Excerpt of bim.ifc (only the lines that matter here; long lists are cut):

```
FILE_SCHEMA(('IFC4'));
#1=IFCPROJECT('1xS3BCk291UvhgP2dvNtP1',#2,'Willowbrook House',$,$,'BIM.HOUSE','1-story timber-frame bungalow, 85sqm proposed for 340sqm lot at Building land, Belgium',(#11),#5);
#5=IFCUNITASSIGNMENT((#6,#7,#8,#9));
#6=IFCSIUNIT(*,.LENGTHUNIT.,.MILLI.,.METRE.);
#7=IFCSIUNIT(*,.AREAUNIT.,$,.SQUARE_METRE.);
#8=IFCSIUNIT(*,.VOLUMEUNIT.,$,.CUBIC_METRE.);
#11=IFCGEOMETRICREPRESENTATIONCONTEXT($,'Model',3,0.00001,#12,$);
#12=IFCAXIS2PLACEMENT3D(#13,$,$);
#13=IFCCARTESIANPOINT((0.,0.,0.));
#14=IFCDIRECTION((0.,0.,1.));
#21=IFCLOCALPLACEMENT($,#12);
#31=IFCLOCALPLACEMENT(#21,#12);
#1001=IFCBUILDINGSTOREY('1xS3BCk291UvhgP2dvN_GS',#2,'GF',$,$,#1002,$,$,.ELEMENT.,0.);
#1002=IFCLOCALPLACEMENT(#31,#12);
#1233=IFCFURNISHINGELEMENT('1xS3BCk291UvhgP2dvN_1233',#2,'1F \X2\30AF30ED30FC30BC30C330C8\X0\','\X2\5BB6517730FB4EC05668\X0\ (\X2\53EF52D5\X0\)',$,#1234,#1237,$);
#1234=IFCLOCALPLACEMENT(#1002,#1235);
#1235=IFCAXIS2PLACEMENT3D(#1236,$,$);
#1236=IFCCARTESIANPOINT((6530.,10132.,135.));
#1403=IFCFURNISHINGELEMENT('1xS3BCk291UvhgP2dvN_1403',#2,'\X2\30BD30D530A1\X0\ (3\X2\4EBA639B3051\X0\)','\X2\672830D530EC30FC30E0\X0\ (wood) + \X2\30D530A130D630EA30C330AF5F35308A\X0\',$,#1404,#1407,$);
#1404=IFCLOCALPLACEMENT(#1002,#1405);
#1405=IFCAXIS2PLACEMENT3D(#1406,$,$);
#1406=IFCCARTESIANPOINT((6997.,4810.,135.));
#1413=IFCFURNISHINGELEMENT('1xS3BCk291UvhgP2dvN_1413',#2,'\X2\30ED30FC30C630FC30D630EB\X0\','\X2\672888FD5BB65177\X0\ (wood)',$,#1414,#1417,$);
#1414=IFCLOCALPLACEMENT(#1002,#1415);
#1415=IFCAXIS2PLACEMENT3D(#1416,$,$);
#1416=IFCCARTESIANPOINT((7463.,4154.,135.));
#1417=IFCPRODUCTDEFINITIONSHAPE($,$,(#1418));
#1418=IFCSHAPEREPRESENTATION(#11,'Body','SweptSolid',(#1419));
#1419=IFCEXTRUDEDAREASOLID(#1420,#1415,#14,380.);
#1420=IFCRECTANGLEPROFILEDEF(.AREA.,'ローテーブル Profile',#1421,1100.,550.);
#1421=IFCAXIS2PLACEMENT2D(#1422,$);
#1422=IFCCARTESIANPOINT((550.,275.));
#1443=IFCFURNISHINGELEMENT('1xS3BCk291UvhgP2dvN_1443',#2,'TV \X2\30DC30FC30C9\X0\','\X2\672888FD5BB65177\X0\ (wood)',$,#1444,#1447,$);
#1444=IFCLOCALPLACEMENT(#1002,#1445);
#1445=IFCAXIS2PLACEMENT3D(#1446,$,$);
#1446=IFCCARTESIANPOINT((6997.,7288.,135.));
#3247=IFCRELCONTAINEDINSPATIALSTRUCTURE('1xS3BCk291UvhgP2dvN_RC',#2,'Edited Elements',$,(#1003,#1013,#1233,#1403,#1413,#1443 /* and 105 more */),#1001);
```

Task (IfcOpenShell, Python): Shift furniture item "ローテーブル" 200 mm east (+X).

```python
import ifcopenshell
import ifcopenshell.api.geometry
import ifcopenshell.util.placement

model = ifcopenshell.open("bim.ifc")

item = model.by_id(1413)
matrix = ifcopenshell.util.placement.get_local_placement(item.ObjectPlacement)
matrix[0, 3] += 200.0
ifcopenshell.api.geometry.edit_object_placement(model, product=item, matrix=matrix, is_si=False)

print(ifcopenshell.util.placement.get_local_placement(item.ObjectPlacement).round(3) + 0.0)

model.write("bim_edited.ifc")
```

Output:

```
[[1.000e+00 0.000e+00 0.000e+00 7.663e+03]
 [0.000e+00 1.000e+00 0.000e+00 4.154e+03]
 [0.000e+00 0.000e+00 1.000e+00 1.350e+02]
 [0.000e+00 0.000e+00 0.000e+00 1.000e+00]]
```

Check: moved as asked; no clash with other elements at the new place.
